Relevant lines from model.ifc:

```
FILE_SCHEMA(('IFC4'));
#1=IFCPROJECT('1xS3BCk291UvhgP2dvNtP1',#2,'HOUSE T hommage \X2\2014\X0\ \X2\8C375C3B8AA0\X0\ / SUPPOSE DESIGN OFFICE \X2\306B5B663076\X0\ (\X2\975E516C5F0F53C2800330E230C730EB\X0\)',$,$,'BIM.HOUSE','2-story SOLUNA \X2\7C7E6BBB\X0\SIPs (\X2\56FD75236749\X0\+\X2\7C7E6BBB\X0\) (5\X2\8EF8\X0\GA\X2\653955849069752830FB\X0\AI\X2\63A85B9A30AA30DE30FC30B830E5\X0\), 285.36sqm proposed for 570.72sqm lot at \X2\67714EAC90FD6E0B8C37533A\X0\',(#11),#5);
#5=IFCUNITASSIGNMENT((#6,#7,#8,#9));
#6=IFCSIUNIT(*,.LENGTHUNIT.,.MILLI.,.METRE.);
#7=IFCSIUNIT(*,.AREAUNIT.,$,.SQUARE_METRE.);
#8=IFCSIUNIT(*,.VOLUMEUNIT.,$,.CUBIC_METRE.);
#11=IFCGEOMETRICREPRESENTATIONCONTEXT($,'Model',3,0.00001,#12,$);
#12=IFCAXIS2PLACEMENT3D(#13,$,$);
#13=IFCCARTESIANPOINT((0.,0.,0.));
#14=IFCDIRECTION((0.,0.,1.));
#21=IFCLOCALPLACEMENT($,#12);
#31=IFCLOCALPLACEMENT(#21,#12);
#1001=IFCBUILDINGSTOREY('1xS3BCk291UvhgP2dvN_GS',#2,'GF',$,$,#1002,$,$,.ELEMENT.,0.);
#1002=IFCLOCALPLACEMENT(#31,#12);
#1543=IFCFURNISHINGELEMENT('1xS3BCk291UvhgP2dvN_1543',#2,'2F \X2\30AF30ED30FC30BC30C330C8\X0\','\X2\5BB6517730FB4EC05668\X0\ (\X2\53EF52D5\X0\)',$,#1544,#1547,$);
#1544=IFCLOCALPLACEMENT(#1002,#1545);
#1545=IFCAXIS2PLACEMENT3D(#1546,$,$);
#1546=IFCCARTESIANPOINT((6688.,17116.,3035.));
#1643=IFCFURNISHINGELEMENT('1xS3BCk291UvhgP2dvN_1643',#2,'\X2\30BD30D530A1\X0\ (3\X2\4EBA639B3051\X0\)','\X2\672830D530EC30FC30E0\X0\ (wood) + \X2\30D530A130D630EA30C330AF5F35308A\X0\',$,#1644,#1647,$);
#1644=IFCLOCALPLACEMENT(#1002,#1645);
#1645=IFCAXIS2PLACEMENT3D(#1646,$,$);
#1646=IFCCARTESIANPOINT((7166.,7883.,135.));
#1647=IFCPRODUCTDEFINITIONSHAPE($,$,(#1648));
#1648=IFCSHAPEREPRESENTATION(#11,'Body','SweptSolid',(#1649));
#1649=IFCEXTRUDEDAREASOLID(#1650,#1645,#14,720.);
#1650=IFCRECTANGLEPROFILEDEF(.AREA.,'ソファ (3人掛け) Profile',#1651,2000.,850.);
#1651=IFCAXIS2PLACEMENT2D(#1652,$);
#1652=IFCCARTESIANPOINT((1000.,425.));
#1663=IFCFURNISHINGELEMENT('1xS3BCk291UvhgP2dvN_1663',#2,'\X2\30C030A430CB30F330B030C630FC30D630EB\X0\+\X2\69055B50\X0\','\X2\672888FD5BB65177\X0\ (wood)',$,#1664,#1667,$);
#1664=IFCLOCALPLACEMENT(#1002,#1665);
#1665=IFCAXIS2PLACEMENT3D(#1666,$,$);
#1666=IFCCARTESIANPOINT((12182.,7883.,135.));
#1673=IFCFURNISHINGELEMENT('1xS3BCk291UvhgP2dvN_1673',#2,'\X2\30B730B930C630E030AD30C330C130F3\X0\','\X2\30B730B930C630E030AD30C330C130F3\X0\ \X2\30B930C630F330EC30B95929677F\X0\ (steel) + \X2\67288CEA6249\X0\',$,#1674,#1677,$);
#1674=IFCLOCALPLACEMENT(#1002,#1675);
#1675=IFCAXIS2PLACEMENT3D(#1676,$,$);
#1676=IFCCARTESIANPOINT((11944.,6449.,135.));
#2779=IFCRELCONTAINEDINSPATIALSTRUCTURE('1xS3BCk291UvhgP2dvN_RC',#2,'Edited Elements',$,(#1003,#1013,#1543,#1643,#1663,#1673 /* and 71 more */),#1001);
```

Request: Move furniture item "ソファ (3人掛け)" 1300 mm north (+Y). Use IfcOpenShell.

```python
import ifcopenshell
import ifcopenshell.api.geometry
import ifcopenshell.util.placement
import ifcopenshell.util.unit

model = ifcopenshell.open("model.ifc")
unit_scale = ifcopenshell.util.unit.calculate_unit_scale(model)

item = model.by_guid("1xS3BCk291UvhgP2dvN_1643")
matrix = ifcopenshell.util.placement.get_local_placement(item.ObjectPlacement)
matrix[1, 3] += 1.3 / unit_scale
ifcopenshell.api.geometry.edit_object_placement(model, product=item, matrix=matrix, is_si=False)

print(ifcopenshell.util.placement.get_local_placement(item.ObjectPlacement).round(3) + 0.0)

model.write("model_rev.ifc")
```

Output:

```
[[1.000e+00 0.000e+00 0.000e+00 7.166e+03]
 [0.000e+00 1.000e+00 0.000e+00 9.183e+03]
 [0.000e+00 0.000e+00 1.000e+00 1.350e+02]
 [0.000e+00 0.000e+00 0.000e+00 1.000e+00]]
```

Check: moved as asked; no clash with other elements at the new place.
